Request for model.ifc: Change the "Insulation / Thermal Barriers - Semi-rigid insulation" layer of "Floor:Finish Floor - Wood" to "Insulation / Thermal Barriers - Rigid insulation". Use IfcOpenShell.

First a look at what the model holds.

```python
import ifcopenshell
import ifcopenshell.util.element

model = ifcopenshell.open("model.ifc")
print(model.schema)
for layer_set in model.by_type("IfcMaterialLayerSet"):
    if layer_set.LayerSetName == "Floor:Finish Floor - Wood":
        for layer in layer_set.MaterialLayers:
            print(layer.id(), layer.Material and layer.Material.Name, layer.LayerThickness, sep=" | ")
        print(len(ifcopenshell.util.element.get_elements_by_material(model, layer_set)), "elements and types use it")
print(sorted(m.Name for m in model.by_type("IfcMaterial") if m.Name)[:60])
```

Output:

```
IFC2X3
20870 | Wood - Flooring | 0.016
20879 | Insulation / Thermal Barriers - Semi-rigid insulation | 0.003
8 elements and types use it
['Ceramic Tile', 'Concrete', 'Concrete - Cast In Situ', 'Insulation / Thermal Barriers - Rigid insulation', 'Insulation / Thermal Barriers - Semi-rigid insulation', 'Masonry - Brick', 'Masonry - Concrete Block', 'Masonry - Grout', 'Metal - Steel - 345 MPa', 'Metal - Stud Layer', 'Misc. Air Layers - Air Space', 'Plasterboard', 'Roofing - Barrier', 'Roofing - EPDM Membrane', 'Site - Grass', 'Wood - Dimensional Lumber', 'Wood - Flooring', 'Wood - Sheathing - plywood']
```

```python
import ifcopenshell
import ifcopenshell.api.material

model = ifcopenshell.open("model.ifc")

layer_set = next(s for s in model.by_type("IfcMaterialLayerSet") if s.LayerSetName == "Floor:Finish Floor - Wood")
layer = next(l for l in layer_set.MaterialLayers if l.Material and l.Material.Name == "Insulation / Thermal Barriers - Semi-rigid insulation")
material = next(m for m in model.by_type("IfcMaterial") if m.Name == "Insulation / Thermal Barriers - Rigid insulation")

# Point this one layer at the other material; renaming the old one would change it everywhere.
ifcopenshell.api.material.edit_layer(model, layer=layer, attributes={}, material=material)

print([l.Material.Name if l.Material else None for l in layer_set.MaterialLayers])

model.write("model_updated.ifc")
```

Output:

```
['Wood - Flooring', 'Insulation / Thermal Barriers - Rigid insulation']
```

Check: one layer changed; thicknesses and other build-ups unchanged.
